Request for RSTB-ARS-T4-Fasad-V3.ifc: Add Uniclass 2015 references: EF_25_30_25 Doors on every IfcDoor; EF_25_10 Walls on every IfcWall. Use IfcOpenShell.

First a look at what the model holds.

```python
import ifcopenshell

model = ifcopenshell.open("RSTB-ARS-T4-Fasad-V3.ifc")
print(model.schema)
print("classifications:", [c.Name for c in model.by_type("IfcClassification")])
for ifc_class in ("IfcDoor", "IfcRoof", "IfcStair", "IfcWall", "IfcWindow"):
    print(ifc_class, len(model.by_type(ifc_class)))
```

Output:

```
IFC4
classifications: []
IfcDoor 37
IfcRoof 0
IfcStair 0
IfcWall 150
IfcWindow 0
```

```python
import ifcopenshell
import ifcopenshell.api.classification

model = ifcopenshell.open("RSTB-ARS-T4-Fasad-V3.ifc")

system = ifcopenshell.api.classification.add_classification(model, classification="Uniclass 2015")

codes = {
    "IfcDoor": ("EF_25_30_25", "Doors"),
    "IfcWall": ("EF_25_10", "Walls"),
}
for ifc_class, (code, name) in codes.items():
    products = model.by_type(ifc_class)
    ifcopenshell.api.classification.add_reference(
        model, products=products, classification=system, identification=code, name=name
    )
    print(code, len(products))

model.write("RSTB-ARS-T4-Fasad-V3_rev.ifc")
```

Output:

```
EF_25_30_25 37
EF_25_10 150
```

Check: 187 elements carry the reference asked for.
